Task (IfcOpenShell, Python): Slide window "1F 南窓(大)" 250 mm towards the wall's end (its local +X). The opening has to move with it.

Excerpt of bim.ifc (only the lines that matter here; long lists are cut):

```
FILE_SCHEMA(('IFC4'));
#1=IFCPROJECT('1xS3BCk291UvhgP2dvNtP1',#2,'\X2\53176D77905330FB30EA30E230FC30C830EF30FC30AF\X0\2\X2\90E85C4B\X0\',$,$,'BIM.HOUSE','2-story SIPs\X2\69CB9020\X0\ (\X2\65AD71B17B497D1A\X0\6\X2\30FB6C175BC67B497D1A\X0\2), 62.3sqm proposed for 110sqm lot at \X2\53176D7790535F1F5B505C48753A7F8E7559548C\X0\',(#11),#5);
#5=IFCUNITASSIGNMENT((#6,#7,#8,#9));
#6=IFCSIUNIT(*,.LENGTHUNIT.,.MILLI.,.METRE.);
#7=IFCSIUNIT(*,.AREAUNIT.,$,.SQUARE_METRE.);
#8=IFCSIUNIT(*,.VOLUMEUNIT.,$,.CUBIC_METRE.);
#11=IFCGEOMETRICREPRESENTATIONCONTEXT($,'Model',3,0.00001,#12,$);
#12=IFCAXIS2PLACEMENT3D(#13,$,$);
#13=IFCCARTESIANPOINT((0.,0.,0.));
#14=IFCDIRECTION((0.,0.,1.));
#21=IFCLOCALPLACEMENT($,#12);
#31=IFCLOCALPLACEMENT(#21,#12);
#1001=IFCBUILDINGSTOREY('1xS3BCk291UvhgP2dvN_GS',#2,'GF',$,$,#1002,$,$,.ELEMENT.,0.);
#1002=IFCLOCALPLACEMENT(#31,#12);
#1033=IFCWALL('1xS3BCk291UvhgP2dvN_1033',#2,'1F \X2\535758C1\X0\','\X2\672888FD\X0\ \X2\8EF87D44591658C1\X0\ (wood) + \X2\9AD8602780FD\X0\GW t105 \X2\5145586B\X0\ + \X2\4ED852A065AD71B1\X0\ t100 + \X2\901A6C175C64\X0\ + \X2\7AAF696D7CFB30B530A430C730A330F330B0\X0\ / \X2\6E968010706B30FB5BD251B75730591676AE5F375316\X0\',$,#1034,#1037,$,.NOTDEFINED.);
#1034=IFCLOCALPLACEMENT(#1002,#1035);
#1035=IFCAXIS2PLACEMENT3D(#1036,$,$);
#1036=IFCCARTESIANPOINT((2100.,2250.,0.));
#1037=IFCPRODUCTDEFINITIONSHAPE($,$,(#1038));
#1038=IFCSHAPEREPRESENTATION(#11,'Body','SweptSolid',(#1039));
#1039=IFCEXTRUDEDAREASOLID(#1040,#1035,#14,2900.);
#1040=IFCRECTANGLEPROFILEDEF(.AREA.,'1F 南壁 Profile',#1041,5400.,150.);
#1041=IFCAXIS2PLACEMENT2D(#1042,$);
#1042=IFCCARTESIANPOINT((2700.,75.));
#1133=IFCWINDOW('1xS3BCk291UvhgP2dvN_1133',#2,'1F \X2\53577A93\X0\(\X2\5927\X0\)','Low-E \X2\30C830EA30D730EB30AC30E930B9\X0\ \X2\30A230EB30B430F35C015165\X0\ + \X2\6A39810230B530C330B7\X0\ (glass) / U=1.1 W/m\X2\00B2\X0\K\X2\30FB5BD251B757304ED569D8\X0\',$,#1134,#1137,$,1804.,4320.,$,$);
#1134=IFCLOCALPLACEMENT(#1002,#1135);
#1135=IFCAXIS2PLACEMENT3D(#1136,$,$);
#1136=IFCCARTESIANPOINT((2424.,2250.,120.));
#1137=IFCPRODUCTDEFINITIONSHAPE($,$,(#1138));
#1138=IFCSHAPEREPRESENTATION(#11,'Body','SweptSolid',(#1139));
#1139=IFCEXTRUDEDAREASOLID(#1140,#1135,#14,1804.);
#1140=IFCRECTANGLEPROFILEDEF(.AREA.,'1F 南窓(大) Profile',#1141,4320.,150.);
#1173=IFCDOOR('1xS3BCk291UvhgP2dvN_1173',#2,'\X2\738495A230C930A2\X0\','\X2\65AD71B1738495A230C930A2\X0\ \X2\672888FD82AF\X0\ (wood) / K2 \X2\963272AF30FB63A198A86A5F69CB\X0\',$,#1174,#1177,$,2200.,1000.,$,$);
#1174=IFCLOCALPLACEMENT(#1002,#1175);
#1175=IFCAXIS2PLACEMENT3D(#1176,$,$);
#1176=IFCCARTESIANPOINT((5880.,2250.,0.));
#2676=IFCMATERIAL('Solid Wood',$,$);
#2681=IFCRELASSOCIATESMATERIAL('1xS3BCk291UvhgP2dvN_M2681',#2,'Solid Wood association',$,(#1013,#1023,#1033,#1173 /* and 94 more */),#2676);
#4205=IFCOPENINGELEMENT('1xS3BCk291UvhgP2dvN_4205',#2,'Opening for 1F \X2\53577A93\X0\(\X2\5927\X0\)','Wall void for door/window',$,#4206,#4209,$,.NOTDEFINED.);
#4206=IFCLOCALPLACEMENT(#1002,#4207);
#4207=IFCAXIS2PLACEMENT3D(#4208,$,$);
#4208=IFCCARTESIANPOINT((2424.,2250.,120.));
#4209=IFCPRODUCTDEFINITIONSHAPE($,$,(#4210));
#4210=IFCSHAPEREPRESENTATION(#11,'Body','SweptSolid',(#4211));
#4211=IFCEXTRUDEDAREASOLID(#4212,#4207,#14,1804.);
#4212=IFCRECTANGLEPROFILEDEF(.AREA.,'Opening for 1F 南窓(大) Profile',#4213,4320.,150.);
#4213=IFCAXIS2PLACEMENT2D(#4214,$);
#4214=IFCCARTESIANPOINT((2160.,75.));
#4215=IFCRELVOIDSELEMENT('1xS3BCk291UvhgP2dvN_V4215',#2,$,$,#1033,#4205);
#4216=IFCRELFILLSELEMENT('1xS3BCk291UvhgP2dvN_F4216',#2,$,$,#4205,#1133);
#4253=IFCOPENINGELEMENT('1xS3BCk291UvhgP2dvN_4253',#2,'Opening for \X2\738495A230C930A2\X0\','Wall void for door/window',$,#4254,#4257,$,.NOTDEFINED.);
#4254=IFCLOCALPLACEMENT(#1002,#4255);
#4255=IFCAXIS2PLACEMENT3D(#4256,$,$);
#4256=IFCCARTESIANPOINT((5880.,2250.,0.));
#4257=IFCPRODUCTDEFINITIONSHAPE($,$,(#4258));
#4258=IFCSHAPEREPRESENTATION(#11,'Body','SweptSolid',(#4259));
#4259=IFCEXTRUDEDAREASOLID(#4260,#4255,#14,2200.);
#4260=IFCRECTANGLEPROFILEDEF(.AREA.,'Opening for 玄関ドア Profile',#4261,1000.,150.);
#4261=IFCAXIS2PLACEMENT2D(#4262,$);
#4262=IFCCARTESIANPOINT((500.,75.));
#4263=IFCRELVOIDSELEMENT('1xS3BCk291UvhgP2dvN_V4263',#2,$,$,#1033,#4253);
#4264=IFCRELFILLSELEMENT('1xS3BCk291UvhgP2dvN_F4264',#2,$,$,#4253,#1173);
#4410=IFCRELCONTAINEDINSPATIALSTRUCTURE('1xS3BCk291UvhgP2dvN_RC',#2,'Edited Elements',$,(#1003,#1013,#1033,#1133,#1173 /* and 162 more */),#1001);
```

```python
import ifcopenshell
import ifcopenshell.api.geometry
import ifcopenshell.util.placement

model = ifcopenshell.open("bim.ifc")

window = model.by_guid("1xS3BCk291UvhgP2dvN_1133")
opening = window.FillsVoids[0].RelatingOpeningElement
wall = opening.VoidsElements[0].RelatingBuildingElement

wall_matrix = ifcopenshell.util.placement.get_local_placement(wall.ObjectPlacement)
shift = wall_matrix[:3, 0] * 250.0
before = ifcopenshell.util.placement.get_local_placement(window.ObjectPlacement)[:3, 3].copy()

# The window is not placed relative to its opening, so move both.
for product in (opening, window):
    matrix = ifcopenshell.util.placement.get_local_placement(product.ObjectPlacement)
    matrix[:3, 3] += shift
    ifcopenshell.api.geometry.edit_object_placement(model, product=product, matrix=matrix, is_si=False)

after = ifcopenshell.util.placement.get_local_placement(window.ObjectPlacement)[:3, 3]
print("window moved by", (after - before).round(3) + 0.0)

model.write("bim_edited.ifc")
```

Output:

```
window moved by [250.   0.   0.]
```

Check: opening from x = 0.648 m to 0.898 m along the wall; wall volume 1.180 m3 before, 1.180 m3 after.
